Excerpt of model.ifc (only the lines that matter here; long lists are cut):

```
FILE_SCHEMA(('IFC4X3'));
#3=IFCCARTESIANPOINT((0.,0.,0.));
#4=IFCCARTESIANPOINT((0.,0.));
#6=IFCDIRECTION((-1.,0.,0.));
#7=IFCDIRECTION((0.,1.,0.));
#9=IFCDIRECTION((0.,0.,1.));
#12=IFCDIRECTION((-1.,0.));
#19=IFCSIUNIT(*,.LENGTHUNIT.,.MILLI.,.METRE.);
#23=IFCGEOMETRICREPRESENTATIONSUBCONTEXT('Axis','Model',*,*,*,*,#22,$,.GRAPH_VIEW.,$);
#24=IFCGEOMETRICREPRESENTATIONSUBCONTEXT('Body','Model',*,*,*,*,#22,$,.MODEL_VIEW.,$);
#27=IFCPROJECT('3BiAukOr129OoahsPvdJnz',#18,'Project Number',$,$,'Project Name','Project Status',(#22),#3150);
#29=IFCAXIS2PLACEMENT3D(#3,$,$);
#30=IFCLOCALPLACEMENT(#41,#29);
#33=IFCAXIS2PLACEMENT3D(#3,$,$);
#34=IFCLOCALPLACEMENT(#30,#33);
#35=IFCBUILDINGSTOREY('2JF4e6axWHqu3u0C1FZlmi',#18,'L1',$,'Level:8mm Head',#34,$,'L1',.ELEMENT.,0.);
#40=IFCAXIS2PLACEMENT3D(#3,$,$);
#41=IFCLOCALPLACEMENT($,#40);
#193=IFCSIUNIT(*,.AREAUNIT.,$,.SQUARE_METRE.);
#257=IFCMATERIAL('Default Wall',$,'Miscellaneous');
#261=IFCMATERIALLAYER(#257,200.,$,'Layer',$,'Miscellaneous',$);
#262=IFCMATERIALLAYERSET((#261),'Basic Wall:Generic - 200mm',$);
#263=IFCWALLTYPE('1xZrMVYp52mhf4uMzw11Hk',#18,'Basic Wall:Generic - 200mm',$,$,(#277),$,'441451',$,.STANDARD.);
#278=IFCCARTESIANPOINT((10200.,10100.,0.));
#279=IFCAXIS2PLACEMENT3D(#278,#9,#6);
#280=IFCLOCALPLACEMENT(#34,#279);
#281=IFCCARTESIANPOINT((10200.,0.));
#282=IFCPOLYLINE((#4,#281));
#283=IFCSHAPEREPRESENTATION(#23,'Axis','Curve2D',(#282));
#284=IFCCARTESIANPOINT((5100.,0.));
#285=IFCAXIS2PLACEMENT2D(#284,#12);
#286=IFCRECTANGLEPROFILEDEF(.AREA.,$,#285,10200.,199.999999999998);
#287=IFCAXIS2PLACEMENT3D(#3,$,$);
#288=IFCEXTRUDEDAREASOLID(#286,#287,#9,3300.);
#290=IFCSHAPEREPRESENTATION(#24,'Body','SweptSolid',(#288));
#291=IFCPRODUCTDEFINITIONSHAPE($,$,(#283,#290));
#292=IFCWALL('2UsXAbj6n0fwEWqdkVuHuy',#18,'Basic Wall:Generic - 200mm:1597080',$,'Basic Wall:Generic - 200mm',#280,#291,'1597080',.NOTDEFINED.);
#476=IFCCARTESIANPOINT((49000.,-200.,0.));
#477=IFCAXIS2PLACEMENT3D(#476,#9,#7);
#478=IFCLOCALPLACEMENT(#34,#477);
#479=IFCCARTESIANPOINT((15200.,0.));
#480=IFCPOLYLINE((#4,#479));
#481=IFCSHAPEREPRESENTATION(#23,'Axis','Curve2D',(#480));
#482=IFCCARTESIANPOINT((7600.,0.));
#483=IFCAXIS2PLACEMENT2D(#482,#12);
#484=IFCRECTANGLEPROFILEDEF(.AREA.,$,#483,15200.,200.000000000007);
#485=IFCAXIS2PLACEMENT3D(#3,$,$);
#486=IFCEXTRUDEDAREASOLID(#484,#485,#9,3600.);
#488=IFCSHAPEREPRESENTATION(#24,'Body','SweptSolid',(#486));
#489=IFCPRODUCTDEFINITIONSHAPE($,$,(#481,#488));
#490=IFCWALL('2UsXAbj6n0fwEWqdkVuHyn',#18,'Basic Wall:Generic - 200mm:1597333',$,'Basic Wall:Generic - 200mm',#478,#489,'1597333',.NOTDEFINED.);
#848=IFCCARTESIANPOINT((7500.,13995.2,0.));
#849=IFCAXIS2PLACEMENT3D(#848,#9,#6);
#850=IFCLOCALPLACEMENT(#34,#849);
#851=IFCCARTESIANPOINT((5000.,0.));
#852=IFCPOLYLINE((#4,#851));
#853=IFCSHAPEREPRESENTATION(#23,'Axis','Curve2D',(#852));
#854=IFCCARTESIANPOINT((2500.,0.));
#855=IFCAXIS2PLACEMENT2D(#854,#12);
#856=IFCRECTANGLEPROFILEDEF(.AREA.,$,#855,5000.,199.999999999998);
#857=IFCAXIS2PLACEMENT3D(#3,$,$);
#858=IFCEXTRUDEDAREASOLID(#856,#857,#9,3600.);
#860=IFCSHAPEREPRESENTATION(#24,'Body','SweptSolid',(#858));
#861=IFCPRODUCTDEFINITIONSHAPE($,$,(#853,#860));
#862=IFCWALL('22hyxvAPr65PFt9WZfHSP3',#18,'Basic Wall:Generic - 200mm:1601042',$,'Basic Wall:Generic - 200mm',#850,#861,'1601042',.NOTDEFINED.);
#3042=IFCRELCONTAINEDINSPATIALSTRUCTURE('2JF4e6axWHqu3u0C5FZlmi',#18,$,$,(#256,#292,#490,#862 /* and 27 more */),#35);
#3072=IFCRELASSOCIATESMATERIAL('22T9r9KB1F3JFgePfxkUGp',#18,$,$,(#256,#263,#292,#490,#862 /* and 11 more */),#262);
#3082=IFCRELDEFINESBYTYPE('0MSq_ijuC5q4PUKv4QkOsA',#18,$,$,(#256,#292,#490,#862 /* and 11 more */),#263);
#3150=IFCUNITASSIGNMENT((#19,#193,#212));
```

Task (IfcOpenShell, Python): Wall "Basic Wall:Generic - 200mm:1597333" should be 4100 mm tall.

```python
import ifcopenshell
import ifcopenshell.geom
import ifcopenshell.util.representation
import ifcopenshell.util.shape
import ifcopenshell.util.unit

model = ifcopenshell.open("model.ifc")
unit_scale = ifcopenshell.util.unit.calculate_unit_scale(model)
settings = ifcopenshell.geom.settings()


def volume(element):
    """Net volume in cubic metres, openings subtracted."""
    shape = ifcopenshell.geom.create_shape(settings, element)
    return ifcopenshell.util.shape.get_volume(shape.geometry)


wall = model.by_id(490)
before = volume(wall)

body = ifcopenshell.util.representation.get_representation(wall, "Model", "Body")
solid = body.Items[0]
old_height = solid.Depth
solid.Depth = 4.1 / unit_scale
after = volume(wall)

print(f"height {old_height:g} -> {solid.Depth:g}, volume {before:.3f} -> {after:.3f} m3")

model.write("model_rev.ifc")
```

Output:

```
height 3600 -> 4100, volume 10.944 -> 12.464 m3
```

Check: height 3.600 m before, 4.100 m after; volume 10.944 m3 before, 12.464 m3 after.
